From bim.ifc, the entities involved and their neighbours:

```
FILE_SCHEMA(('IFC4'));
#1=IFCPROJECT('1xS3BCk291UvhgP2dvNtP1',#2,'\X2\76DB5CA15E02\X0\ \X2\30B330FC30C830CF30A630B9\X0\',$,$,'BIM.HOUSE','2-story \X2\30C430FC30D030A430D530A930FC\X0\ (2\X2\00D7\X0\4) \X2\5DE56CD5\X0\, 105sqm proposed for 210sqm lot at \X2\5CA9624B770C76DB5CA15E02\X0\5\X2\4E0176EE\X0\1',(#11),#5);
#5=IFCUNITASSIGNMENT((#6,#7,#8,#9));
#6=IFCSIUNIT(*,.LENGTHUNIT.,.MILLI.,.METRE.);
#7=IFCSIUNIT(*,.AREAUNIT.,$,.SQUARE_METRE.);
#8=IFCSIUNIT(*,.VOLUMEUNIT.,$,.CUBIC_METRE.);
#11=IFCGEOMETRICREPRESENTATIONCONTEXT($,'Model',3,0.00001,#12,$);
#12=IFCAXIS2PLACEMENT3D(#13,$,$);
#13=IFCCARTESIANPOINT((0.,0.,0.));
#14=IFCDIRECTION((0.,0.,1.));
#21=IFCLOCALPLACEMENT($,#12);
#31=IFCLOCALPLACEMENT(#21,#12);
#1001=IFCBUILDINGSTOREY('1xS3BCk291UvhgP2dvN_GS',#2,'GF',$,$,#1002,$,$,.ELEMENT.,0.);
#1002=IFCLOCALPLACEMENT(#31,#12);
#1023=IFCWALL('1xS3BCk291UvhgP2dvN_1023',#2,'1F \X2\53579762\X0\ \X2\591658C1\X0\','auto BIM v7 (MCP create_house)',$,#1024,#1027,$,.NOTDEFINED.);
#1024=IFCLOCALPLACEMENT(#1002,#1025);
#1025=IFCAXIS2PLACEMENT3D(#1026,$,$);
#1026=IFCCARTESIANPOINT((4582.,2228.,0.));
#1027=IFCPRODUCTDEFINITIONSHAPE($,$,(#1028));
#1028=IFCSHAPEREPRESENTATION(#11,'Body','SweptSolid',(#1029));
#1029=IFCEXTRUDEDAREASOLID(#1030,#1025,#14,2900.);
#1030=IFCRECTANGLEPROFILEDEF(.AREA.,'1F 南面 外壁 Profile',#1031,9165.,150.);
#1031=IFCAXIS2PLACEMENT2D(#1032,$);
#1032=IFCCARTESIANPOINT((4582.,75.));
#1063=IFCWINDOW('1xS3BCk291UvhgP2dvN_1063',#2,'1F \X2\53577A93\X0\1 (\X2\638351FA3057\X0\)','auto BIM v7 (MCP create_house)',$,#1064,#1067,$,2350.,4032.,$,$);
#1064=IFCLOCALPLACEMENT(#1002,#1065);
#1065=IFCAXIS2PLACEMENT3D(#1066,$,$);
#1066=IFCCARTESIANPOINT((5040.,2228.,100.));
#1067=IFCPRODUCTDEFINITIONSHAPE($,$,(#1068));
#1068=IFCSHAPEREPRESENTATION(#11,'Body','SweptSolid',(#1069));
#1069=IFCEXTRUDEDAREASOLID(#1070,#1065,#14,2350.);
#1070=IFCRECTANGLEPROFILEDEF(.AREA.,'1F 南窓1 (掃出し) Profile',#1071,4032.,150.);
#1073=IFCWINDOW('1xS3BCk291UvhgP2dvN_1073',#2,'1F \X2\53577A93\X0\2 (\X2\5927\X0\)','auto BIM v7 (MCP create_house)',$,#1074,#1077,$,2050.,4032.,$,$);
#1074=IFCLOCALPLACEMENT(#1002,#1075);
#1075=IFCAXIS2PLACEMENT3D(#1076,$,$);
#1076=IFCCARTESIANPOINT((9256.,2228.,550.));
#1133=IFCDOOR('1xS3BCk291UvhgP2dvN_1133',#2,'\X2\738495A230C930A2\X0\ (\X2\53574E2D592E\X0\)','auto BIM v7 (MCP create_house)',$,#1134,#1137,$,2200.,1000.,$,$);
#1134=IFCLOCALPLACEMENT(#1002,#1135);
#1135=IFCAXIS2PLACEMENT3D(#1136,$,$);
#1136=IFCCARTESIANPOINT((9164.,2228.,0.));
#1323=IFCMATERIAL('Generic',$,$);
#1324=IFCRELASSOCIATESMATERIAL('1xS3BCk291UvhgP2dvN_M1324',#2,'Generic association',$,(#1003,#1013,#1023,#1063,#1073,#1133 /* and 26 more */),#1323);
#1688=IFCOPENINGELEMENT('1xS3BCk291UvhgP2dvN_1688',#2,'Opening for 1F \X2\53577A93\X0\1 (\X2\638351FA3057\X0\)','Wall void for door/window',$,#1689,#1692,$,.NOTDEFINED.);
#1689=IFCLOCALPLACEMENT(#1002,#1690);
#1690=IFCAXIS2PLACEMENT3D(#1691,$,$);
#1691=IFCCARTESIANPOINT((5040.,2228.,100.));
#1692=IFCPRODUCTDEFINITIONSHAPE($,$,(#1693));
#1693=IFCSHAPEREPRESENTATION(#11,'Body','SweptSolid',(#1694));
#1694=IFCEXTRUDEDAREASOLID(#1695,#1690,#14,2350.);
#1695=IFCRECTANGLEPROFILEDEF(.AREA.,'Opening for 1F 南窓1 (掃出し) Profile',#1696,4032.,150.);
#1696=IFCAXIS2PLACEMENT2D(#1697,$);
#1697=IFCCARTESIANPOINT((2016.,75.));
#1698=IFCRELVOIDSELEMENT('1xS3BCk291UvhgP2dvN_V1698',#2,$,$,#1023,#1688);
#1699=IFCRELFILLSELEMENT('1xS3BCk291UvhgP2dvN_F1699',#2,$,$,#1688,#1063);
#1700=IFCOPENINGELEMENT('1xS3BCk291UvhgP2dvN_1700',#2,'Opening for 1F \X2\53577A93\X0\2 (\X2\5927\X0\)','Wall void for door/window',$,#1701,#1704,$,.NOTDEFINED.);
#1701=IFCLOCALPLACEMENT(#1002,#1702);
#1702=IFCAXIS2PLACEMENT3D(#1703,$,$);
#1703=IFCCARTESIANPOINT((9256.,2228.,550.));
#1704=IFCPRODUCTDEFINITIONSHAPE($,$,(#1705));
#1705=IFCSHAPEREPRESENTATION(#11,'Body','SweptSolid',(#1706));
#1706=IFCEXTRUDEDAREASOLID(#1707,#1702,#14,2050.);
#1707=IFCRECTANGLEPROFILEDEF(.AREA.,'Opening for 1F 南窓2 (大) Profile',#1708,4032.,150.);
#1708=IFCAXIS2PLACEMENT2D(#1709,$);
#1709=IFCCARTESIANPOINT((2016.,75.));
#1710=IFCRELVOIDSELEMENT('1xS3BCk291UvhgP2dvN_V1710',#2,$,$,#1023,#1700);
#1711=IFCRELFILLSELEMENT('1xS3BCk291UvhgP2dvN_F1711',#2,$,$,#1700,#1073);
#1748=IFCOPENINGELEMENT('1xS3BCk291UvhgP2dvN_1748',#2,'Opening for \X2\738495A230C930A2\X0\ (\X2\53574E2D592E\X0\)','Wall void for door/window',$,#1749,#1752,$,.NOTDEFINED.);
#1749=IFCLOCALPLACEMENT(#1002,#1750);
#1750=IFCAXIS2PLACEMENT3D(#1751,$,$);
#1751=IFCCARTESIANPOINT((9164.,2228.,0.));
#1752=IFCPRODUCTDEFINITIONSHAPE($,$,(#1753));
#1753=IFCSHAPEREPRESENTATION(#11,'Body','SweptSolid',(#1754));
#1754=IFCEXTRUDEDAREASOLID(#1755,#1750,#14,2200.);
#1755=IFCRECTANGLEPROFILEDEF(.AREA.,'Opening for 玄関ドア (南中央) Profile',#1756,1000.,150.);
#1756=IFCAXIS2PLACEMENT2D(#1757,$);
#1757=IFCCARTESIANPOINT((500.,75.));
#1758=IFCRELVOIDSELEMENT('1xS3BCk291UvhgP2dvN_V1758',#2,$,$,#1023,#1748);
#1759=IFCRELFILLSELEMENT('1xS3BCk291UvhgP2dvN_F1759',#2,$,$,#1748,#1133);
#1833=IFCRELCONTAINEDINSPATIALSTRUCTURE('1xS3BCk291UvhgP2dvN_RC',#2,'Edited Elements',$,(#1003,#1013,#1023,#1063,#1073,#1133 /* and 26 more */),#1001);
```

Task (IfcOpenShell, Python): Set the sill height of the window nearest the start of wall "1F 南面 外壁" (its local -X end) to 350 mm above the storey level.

```python
import numpy as np
import ifcopenshell
import ifcopenshell.api.geometry
import ifcopenshell.geom
import ifcopenshell.util.element
import ifcopenshell.util.placement
import ifcopenshell.util.shape
import ifcopenshell.util.unit

model = ifcopenshell.open("bim.ifc")
unit_scale = ifcopenshell.util.unit.calculate_unit_scale(model)

window = model.by_guid("1xS3BCk291UvhgP2dvN_1063")
opening = window.FillsVoids[0].RelatingOpeningElement
storey = ifcopenshell.util.element.get_container(window, ifc_class="IfcBuildingStorey")
level = ifcopenshell.util.placement.get_local_placement(storey.ObjectPlacement)[2, 3]

# The opening's origin need not be at the sill, so measure its lowest point.
shape = ifcopenshell.geom.create_shape(ifcopenshell.geom.settings(), opening)
bottom = ifcopenshell.util.shape.get_shape_bottom_elevation(shape, shape.geometry) / unit_scale
dz = level + 0.35 / unit_scale - bottom

shift = np.array([0.0, 0.0, dz])
# The window is not placed relative to its opening, so move both.
for product in (opening, window):
    matrix = ifcopenshell.util.placement.get_local_placement(product.ObjectPlacement)
    matrix[:3, 3] += shift
    ifcopenshell.api.geometry.edit_object_placement(model, product=product, matrix=matrix, is_si=False)

print(f"moved by {dz * unit_scale:+.3f} m")

model.write("bim_v2.ifc")
```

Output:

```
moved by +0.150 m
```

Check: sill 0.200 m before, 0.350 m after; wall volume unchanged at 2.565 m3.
